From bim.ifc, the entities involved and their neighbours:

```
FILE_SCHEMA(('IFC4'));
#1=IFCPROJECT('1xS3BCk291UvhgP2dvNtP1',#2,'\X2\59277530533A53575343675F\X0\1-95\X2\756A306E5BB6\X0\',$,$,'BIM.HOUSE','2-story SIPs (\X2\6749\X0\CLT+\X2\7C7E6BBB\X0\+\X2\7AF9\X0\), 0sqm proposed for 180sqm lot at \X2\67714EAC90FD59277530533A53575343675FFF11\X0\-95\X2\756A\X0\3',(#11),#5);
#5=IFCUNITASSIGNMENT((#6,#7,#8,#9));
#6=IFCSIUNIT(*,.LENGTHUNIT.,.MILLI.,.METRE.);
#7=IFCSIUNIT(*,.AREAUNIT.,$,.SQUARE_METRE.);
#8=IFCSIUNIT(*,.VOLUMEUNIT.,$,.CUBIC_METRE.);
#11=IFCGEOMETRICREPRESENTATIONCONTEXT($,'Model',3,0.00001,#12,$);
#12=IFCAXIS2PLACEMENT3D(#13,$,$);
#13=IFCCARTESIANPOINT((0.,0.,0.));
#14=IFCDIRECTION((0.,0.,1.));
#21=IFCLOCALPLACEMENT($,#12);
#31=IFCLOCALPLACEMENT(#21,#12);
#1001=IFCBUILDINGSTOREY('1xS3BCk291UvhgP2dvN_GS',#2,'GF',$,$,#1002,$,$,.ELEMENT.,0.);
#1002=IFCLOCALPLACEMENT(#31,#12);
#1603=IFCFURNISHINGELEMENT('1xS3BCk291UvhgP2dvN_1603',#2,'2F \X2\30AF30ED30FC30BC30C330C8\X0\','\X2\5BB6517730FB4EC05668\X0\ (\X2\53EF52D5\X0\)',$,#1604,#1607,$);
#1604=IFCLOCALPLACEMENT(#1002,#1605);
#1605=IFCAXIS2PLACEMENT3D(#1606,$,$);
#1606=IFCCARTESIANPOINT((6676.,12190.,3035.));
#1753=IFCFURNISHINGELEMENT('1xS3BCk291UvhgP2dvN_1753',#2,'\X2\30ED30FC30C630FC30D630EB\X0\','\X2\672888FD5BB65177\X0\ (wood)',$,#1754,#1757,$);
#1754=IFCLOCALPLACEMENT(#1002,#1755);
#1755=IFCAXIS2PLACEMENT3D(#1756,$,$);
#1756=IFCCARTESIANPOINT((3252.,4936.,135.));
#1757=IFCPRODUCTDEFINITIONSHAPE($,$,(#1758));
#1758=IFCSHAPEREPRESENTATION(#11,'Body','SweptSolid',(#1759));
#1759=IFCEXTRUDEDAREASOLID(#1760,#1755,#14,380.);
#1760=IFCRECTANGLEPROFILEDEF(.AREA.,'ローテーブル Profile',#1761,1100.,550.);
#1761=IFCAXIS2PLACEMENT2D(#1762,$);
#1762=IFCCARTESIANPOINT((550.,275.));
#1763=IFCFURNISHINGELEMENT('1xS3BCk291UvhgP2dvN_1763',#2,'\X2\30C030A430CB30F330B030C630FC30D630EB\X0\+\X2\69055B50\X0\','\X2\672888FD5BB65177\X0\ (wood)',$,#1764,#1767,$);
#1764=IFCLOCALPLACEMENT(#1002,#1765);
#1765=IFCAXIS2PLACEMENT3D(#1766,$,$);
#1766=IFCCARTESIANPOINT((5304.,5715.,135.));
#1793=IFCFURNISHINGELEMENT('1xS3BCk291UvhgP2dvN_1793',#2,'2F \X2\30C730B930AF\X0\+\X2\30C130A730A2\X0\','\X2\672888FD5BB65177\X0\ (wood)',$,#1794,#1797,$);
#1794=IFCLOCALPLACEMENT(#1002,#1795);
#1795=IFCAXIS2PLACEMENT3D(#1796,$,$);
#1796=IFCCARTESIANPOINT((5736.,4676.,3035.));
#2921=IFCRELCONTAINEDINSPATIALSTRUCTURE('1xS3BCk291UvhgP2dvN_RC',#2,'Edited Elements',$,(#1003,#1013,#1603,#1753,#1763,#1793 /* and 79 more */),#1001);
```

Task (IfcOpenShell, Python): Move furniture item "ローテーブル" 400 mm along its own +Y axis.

```python
import ifcopenshell
import ifcopenshell.api.geometry
import ifcopenshell.util.placement
import ifcopenshell.util.unit

model = ifcopenshell.open("bim.ifc")
unit_scale = ifcopenshell.util.unit.calculate_unit_scale(model)

item = model.by_guid("1xS3BCk291UvhgP2dvN_1753")
matrix = ifcopenshell.util.placement.get_local_placement(item.ObjectPlacement)
matrix[:3, 3] += matrix[:3, 1] * 0.4 / unit_scale
ifcopenshell.api.geometry.edit_object_placement(model, product=item, matrix=matrix, is_si=False)

print(ifcopenshell.util.placement.get_local_placement(item.ObjectPlacement).round(3) + 0.0)

model.write("bim-out.ifc")
```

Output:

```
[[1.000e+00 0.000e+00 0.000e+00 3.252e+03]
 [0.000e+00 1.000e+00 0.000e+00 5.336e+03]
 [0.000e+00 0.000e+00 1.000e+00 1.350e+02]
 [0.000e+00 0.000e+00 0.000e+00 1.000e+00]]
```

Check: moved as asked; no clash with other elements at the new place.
